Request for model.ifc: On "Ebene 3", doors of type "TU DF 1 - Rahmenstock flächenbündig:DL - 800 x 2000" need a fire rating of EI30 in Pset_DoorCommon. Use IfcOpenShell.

First a look at what the model holds.

```python
import ifcopenshell
import ifcopenshell.util.element

model = ifcopenshell.open("model.ifc")
print(model.schema)
storey = next(s for s in model.by_type("IfcBuildingStorey") if s.Name == "Ebene 3")
doors = [e for e in ifcopenshell.util.element.get_decomposition(storey) if e.is_a("IfcDoor")]
seen = {}
for e in doors:
    element_type = ifcopenshell.util.element.get_type(e)
    key = (element_type.Name if element_type != e and element_type else None, ifcopenshell.util.element.get_pset(e, "Pset_DoorCommon", "FireRating"))
    seen[key] = seen.get(key, 0) + 1
for (name, value), count in sorted(seen.items(), key=str):
    print(count, "x", name, "|", value)
```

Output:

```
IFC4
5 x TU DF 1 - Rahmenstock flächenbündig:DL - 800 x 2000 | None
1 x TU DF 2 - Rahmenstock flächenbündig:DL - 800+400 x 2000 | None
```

```python
import ifcopenshell
import ifcopenshell.api.pset
import ifcopenshell.util.element

model = ifcopenshell.open("model.ifc")

storey = next(s for s in model.by_type("IfcBuildingStorey") if s.Name == "Ebene 3")
doors = [e for e in ifcopenshell.util.element.get_decomposition(storey) if e.is_a("IfcDoor")]

count = 0
for e in doors:
    element_type = ifcopenshell.util.element.get_type(e)
    if element_type in (None, e) or element_type.Name != "TU DF 1 - Rahmenstock flächenbündig:DL - 800 x 2000":
        continue
    # add_pset returns the element's existing set when there is one.
    pset = ifcopenshell.api.pset.add_pset(model, product=e, name="Pset_DoorCommon")
    ifcopenshell.api.pset.edit_pset(model, pset=pset, properties={"FireRating": "EI30"})
    count += 1

print(count, "doors updated")

model.write("model_updated.ifc")
```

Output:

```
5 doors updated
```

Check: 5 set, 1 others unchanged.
